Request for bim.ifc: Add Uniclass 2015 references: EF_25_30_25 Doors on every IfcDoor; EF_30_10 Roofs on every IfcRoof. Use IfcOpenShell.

First a look at what the model holds.

```python
import ifcopenshell

model = ifcopenshell.open("bim.ifc")
print(model.schema)
print("classifications:", [c.Name for c in model.by_type("IfcClassification")])
for ifc_class in ("IfcDoor", "IfcRoof", "IfcStair", "IfcWall", "IfcWindow"):
    print(ifc_class, len(model.by_type(ifc_class)))
```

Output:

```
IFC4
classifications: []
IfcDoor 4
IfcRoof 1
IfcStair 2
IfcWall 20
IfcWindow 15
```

```python
import ifcopenshell
import ifcopenshell.api.classification

model = ifcopenshell.open("bim.ifc")

system = ifcopenshell.api.classification.add_classification(model, classification="Uniclass 2015")

codes = {
    "IfcDoor": ("EF_25_30_25", "Doors"),
    "IfcRoof": ("EF_30_10", "Roofs"),
}
for ifc_class, (code, name) in codes.items():
    products = model.by_type(ifc_class)
    ifcopenshell.api.classification.add_reference(
        model, products=products, classification=system, identification=code, name=name
    )
    print(code, len(products))

model.write("bim_edited.ifc")
```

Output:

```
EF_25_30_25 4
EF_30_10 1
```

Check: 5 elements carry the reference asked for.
